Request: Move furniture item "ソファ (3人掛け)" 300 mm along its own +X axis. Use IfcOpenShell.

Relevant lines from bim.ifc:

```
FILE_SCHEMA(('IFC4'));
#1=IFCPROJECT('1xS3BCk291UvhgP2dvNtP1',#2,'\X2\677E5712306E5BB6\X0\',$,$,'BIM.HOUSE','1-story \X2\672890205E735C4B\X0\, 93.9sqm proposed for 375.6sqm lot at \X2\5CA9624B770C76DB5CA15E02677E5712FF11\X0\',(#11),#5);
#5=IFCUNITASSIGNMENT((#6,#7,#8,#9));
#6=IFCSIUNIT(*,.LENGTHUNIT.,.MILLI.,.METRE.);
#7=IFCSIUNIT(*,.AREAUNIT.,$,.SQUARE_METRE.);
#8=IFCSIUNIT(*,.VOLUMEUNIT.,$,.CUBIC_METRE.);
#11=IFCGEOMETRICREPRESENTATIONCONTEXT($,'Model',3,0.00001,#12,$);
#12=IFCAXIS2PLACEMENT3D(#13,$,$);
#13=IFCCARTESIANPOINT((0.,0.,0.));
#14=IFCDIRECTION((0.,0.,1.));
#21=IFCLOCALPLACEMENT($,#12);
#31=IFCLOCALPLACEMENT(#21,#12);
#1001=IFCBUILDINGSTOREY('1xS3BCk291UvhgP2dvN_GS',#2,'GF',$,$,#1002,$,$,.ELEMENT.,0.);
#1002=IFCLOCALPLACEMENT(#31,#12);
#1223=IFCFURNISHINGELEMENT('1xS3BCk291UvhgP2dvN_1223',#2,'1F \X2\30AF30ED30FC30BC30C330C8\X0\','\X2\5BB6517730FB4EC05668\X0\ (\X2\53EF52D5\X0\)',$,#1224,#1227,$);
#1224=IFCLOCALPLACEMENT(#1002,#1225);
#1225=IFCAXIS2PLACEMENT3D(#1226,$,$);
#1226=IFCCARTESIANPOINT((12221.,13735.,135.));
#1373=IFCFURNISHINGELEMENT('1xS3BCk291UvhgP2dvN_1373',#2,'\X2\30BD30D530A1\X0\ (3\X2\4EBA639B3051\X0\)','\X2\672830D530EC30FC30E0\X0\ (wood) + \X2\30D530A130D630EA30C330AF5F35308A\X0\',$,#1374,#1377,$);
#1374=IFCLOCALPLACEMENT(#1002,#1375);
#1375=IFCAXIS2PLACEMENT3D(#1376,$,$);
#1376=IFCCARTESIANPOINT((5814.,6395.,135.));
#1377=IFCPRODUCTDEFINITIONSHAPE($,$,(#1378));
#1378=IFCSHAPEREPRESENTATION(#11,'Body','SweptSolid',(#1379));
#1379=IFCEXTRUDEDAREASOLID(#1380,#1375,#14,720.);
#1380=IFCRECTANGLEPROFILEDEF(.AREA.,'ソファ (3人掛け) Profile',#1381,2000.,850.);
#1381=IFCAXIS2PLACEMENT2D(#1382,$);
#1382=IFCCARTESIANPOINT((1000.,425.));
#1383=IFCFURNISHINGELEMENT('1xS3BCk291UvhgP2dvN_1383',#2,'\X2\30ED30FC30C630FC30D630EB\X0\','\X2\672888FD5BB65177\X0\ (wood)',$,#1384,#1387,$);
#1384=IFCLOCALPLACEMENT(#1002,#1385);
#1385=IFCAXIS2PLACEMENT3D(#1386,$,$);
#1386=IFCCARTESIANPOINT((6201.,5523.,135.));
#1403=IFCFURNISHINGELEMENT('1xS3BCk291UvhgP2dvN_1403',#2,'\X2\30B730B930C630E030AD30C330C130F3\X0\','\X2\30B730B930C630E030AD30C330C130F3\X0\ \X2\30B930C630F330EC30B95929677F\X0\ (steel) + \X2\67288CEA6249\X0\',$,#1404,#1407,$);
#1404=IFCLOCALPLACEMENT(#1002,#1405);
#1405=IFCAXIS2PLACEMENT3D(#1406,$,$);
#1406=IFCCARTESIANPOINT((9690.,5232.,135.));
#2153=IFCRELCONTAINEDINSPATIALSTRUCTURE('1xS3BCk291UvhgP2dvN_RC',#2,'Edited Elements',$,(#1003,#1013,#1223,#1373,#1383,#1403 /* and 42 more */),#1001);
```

```python
import ifcopenshell
import ifcopenshell.api.geometry
import ifcopenshell.util.placement

model = ifcopenshell.open("bim.ifc")

item = model.by_id(1373)
matrix = ifcopenshell.util.placement.get_local_placement(item.ObjectPlacement)
matrix[:3, 3] += matrix[:3, 0] * 300.0
ifcopenshell.api.geometry.edit_object_placement(model, product=item, matrix=matrix, is_si=False)

print(ifcopenshell.util.placement.get_local_placement(item.ObjectPlacement).round(3) + 0.0)

model.write("bim_v2.ifc")
```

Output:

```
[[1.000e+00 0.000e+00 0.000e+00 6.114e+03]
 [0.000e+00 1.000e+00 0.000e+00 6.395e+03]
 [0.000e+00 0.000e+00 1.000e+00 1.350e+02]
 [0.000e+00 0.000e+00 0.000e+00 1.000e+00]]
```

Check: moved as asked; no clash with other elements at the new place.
